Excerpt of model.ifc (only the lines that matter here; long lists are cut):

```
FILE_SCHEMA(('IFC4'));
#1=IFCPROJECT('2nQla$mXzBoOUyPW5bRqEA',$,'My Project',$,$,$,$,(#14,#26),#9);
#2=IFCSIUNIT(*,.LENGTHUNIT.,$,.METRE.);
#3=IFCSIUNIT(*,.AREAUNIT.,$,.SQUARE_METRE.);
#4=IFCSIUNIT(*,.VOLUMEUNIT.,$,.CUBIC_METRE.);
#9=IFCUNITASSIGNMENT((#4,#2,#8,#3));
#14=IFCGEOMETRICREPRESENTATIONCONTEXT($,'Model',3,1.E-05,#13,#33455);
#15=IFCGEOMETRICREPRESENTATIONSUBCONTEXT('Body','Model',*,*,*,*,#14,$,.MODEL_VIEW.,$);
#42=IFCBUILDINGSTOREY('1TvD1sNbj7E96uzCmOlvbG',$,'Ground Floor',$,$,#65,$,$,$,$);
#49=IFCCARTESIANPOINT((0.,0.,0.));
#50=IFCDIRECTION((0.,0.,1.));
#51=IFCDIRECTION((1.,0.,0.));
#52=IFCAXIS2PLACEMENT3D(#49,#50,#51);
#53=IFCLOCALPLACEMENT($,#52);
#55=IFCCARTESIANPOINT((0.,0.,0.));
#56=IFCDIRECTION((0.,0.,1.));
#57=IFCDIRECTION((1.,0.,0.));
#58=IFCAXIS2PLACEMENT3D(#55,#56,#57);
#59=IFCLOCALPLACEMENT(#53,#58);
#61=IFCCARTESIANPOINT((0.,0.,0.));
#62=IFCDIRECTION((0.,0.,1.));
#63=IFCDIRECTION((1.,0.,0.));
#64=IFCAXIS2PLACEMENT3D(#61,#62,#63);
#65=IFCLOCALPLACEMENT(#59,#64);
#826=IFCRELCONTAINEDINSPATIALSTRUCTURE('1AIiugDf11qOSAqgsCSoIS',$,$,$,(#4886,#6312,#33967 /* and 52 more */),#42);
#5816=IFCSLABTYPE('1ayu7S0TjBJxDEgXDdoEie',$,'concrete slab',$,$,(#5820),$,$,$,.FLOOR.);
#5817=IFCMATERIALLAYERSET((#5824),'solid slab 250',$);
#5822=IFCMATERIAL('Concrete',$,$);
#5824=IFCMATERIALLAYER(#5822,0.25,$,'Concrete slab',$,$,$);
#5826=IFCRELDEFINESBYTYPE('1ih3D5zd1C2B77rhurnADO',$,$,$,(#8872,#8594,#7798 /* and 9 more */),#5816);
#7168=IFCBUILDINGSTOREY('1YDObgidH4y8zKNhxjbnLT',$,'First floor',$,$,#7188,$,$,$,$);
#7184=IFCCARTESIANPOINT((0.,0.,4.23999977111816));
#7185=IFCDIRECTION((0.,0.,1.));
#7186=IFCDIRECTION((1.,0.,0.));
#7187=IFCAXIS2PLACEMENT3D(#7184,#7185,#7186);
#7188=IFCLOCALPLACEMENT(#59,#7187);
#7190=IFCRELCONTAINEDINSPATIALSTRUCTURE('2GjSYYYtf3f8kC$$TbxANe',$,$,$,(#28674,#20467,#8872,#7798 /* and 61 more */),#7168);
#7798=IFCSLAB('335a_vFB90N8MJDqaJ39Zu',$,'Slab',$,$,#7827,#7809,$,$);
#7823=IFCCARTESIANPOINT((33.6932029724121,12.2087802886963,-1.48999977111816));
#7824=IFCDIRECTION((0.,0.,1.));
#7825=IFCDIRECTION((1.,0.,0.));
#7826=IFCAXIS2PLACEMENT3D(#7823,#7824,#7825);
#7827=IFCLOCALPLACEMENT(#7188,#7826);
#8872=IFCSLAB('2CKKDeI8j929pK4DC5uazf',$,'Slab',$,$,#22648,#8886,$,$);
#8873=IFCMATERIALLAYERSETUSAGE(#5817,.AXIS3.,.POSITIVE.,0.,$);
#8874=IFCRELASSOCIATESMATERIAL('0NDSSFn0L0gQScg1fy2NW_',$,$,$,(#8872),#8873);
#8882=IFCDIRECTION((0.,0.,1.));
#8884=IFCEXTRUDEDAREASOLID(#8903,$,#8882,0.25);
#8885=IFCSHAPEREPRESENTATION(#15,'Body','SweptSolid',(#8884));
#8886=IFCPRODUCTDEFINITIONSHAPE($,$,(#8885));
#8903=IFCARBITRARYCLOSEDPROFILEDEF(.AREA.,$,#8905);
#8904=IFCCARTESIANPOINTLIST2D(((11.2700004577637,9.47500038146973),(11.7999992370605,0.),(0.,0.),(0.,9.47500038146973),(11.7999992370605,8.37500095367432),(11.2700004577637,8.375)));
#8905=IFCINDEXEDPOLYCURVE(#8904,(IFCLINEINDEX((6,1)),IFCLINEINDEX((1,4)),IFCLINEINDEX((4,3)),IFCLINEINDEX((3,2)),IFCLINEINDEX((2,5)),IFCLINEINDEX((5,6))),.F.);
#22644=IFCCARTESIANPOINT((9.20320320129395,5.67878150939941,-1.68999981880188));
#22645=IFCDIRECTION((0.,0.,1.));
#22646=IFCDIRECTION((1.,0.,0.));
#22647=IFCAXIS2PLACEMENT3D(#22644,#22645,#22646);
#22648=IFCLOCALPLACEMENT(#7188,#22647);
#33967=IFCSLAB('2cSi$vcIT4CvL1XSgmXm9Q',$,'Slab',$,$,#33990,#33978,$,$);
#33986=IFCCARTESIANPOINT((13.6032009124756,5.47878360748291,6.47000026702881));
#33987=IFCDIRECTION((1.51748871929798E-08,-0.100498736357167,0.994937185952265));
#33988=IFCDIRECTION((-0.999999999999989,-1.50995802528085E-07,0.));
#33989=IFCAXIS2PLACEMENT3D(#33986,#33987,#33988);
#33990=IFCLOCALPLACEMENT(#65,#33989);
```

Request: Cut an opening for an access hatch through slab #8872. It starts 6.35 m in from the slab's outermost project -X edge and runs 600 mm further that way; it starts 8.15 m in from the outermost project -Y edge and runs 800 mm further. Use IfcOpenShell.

```python
import numpy as np
import ifcopenshell
import ifcopenshell.api.feature
import ifcopenshell.api.geometry
import ifcopenshell.api.root
import ifcopenshell.geom
import ifcopenshell.util.placement
import ifcopenshell.util.representation
import ifcopenshell.util.shape
import ifcopenshell.util.unit

model = ifcopenshell.open("model.ifc")
unit_scale = ifcopenshell.util.unit.calculate_unit_scale(model)
settings = ifcopenshell.geom.settings()


def volume(element):
    """Net volume in cubic metres, openings subtracted."""
    shape = ifcopenshell.geom.create_shape(settings, element)
    return ifcopenshell.util.shape.get_volume(shape.geometry)


slab = model.by_guid("2CKKDeI8j929pK4DC5uazf")
before = volume(slab)

# Extent in the slab's own axes, in metres. The edges named are its -X and -Y sides.
slab_shape = ifcopenshell.geom.create_shape(settings, slab)
vertices = ifcopenshell.util.shape.get_vertices(slab_shape.geometry)
x_min, y_min, bottom = vertices.min(axis=0)
top = vertices[:, 2].max()

opening = ifcopenshell.api.root.create_entity(model, ifc_class="IfcOpeningElement", name="Access hatch opening", predefined_type="OPENING")
context = ifcopenshell.util.representation.get_context(model, "Model", "Body", "MODEL_VIEW")
width, depth = 0.6, 0.8
outline = [(0.0, 0.0), (width, 0.0), (width, depth), (0.0, depth), (0.0, 0.0)]
# Overshoot both faces by 50 mm so the cut is clean.
shape = ifcopenshell.api.geometry.add_slab_representation(
    model, context=context, depth=top - bottom + 0.1, polyline=outline
)
ifcopenshell.api.geometry.assign_representation(model, product=opening, representation=shape)

matrix = ifcopenshell.util.placement.get_local_placement(slab.ObjectPlacement)
matrix[:, 3] = matrix @ np.append(np.array([x_min + 6.35, y_min + 8.15, bottom - 0.05]) / unit_scale, 1.0)
ifcopenshell.api.geometry.edit_object_placement(model, product=opening, matrix=matrix, is_si=False)
ifcopenshell.api.feature.add_feature(model, feature=opening, element=slab)

after = volume(slab)

print(f"slab volume {before:.3f} -> {after:.3f} m3")

model.write("model_edited.ifc")
```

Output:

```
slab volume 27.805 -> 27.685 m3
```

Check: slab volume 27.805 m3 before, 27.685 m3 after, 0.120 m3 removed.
